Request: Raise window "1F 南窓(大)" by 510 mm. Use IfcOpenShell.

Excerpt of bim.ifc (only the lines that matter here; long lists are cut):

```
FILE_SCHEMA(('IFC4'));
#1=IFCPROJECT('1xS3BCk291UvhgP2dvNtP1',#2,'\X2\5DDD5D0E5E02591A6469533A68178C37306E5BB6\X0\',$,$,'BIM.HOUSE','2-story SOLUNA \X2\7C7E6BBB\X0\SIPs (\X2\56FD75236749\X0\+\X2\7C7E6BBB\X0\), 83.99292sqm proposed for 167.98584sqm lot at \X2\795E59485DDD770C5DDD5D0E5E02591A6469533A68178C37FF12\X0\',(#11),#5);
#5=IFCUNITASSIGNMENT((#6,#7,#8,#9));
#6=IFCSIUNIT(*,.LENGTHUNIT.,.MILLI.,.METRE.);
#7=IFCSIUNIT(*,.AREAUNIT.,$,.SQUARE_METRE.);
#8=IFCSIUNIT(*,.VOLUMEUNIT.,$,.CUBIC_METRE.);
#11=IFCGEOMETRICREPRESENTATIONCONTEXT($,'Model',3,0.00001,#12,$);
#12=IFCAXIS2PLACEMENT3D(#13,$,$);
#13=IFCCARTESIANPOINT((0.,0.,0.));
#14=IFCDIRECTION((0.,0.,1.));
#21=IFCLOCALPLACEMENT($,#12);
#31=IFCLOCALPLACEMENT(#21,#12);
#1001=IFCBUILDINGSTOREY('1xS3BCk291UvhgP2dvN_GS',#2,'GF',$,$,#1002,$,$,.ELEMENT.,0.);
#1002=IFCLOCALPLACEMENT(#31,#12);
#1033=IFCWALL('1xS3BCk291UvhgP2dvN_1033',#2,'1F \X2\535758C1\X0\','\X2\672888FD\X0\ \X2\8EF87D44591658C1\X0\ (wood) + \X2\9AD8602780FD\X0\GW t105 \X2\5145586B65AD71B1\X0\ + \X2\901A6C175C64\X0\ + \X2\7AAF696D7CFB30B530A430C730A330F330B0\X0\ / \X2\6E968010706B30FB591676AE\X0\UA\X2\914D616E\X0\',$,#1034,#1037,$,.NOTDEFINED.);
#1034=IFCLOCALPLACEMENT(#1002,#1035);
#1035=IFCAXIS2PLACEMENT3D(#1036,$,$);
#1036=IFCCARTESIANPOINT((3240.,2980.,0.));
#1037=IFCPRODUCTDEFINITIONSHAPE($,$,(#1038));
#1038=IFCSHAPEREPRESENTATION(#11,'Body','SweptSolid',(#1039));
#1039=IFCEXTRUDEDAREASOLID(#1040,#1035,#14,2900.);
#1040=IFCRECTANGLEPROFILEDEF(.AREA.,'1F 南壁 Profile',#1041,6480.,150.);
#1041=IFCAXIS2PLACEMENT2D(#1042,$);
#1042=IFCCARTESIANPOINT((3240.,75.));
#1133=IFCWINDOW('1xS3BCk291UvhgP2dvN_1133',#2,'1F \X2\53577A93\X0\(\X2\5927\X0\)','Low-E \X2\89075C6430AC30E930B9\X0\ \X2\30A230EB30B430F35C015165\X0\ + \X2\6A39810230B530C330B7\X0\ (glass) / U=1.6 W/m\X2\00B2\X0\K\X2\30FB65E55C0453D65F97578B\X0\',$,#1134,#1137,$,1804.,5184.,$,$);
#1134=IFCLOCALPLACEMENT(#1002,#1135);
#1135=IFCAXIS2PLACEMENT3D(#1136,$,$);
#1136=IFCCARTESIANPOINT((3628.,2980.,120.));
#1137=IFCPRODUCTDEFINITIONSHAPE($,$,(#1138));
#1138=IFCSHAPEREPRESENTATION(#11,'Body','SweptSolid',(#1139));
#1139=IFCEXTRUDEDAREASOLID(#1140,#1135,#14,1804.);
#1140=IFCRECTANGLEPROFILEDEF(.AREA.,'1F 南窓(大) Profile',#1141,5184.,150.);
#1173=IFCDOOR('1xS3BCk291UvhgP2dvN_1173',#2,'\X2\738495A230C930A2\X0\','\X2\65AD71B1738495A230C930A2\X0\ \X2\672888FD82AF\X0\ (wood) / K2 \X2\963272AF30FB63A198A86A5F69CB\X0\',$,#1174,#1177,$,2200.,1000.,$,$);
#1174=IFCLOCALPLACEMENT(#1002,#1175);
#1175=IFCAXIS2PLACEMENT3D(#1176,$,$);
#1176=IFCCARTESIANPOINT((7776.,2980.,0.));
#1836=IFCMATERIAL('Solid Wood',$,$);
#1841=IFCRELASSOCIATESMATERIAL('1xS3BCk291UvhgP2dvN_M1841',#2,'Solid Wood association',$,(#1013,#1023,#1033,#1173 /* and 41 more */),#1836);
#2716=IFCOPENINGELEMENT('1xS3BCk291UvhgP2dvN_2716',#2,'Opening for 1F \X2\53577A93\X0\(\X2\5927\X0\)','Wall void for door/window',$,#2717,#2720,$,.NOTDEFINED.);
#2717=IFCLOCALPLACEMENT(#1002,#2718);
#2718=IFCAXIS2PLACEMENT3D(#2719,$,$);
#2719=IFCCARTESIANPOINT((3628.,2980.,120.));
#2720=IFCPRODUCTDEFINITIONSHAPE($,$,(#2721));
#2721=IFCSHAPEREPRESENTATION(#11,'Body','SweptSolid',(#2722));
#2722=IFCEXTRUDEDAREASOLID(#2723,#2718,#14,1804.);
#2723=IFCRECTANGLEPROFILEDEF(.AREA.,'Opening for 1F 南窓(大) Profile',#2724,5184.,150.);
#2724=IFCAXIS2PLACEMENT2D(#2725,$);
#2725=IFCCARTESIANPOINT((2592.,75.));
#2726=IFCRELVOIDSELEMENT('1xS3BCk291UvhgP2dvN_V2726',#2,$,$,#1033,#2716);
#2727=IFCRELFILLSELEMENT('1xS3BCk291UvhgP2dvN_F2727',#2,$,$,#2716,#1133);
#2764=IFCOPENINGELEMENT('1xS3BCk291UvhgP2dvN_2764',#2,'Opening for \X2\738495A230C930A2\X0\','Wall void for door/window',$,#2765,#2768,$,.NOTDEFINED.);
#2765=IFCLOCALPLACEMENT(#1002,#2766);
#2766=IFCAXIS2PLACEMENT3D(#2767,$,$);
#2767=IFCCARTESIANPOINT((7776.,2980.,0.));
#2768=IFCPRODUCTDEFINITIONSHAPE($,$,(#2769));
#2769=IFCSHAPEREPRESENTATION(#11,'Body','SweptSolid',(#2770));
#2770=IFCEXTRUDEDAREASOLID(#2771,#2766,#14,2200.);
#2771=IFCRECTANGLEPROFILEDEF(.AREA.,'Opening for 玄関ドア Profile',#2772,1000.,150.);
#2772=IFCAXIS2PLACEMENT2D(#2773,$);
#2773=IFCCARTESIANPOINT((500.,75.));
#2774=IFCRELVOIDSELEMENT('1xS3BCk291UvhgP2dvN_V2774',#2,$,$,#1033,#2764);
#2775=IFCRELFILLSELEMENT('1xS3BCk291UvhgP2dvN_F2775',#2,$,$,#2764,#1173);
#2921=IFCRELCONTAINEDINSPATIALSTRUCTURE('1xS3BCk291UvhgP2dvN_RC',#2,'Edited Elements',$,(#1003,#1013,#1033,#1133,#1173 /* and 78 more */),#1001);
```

```python
import numpy as np
import ifcopenshell
import ifcopenshell.api.geometry
import ifcopenshell.util.placement
import ifcopenshell.util.unit

model = ifcopenshell.open("bim.ifc")
unit_scale = ifcopenshell.util.unit.calculate_unit_scale(model)

window = model.by_id(1133)
opening = window.FillsVoids[0].RelatingOpeningElement
dz = 0.51 / unit_scale

shift = np.array([0.0, 0.0, dz])
# The window is not placed relative to its opening, so move both.
for product in (opening, window):
    matrix = ifcopenshell.util.placement.get_local_placement(product.ObjectPlacement)
    matrix[:3, 3] += shift
    ifcopenshell.api.geometry.edit_object_placement(model, product=product, matrix=matrix, is_si=False)

print(f"moved by {dz * unit_scale:+.3f} m")

model.write("bim-out.ifc")
```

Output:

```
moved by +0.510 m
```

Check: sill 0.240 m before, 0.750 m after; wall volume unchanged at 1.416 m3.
